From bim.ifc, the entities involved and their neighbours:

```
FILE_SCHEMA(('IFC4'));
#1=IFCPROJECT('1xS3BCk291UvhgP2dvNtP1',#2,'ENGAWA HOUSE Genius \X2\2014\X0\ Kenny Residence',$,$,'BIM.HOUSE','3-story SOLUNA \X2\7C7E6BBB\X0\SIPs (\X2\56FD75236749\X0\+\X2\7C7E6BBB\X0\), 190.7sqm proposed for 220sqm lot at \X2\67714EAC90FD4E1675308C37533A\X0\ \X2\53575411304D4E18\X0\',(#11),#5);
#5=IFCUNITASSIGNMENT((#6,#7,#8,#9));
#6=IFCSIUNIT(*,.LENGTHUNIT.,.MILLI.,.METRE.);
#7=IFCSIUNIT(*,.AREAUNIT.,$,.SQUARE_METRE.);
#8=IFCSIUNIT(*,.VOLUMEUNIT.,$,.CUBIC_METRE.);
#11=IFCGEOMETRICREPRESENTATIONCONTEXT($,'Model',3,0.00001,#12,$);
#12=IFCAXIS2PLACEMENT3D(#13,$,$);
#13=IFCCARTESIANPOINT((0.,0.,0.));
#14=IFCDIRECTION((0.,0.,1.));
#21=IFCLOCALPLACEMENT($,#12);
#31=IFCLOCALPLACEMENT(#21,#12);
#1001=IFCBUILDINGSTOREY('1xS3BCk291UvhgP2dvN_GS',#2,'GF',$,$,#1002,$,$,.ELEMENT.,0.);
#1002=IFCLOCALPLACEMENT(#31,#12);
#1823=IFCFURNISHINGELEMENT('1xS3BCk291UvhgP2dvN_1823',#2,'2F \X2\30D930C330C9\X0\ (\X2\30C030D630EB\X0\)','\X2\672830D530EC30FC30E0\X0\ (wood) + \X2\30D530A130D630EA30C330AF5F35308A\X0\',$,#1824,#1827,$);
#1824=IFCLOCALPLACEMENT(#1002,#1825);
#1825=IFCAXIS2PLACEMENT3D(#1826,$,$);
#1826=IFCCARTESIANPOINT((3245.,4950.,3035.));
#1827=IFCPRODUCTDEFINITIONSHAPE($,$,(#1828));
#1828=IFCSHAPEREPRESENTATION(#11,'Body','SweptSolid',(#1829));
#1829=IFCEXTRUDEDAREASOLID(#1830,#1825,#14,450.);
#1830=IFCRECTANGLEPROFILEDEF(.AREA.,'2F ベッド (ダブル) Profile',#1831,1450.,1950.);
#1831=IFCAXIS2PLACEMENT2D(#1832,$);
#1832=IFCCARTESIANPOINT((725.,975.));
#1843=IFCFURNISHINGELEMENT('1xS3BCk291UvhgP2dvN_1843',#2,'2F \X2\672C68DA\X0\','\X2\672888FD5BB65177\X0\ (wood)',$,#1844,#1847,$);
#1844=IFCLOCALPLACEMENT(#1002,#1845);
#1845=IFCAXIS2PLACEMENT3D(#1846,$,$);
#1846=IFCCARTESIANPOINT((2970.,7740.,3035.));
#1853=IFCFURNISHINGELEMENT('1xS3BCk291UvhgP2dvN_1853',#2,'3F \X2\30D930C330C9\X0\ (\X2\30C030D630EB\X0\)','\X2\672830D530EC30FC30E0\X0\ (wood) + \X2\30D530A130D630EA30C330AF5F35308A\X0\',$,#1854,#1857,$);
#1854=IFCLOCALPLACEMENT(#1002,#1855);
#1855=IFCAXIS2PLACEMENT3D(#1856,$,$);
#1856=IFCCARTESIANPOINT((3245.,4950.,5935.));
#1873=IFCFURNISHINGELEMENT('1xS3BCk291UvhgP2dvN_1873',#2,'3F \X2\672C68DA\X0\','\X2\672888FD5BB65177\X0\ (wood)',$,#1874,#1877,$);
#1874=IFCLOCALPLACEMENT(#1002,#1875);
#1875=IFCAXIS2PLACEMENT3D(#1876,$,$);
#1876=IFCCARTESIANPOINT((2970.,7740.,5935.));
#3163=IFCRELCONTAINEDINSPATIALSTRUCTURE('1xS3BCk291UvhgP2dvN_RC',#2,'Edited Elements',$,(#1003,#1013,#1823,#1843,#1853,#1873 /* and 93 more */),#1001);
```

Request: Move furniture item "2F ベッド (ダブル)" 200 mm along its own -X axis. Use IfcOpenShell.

```python
import ifcopenshell
import ifcopenshell.api.geometry
import ifcopenshell.util.placement
import ifcopenshell.util.unit

model = ifcopenshell.open("bim.ifc")
unit_scale = ifcopenshell.util.unit.calculate_unit_scale(model)

item = model.by_guid("1xS3BCk291UvhgP2dvN_1823")
matrix = ifcopenshell.util.placement.get_local_placement(item.ObjectPlacement)
matrix[:3, 3] -= matrix[:3, 0] * 0.2 / unit_scale
ifcopenshell.api.geometry.edit_object_placement(model, product=item, matrix=matrix, is_si=False)

print(ifcopenshell.util.placement.get_local_placement(item.ObjectPlacement).round(3) + 0.0)

model.write("bim_rev.ifc")
```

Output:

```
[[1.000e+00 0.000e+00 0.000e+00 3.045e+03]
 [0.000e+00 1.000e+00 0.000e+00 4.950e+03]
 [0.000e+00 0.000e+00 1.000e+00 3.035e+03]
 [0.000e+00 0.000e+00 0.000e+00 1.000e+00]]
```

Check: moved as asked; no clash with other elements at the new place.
